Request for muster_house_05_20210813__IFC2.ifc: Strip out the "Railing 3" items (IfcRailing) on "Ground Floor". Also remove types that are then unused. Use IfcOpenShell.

First a look at what the model holds.

```python
import ifcopenshell
import ifcopenshell.util.element

model = ifcopenshell.open("muster_house_05_20210813__IFC2.ifc")
print(model.schema)
storey = next(s for s in model.by_type("IfcBuildingStorey") if s.Name == "Ground Floor")
railings = [e for e in ifcopenshell.util.element.get_decomposition(storey) if e.is_a("IfcRailing")]
seen = {}
for e in railings:
    element_type = ifcopenshell.util.element.get_type(e)
    name = element_type.Name if element_type not in (None, e) else None
    seen[name] = seen.get(name, 0) + 1
for name, count in sorted(seen.items(), key=str):
    print(count, "x", name)
```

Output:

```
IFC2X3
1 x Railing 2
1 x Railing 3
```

```python
import ifcopenshell
import ifcopenshell.api.root
import ifcopenshell.util.element

model = ifcopenshell.open("muster_house_05_20210813__IFC2.ifc")

storey = next(s for s in model.by_type("IfcBuildingStorey") if s.Name == "Ground Floor")
railings = [e for e in ifcopenshell.util.element.get_decomposition(storey) if e.is_a("IfcRailing")]
targets = [e for e in railings if (t := ifcopenshell.util.element.get_type(e)) not in (None, e) and t.Name == "Railing 3"]
types = {ifcopenshell.util.element.get_type(e) for e in targets} - {None, *targets}

for e in targets:
    ifcopenshell.api.root.remove_product(model, product=e)
print(len(targets), "removed")

unused = [t for t in types if not ifcopenshell.util.element.get_types(t)]
for t in unused:
    ifcopenshell.api.root.remove_product(model, product=t)
print(len(unused), "unused types removed")

model.write("muster_house_05_20210813__IFC2_v2.ifc")
```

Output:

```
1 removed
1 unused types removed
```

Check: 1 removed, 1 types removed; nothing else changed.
